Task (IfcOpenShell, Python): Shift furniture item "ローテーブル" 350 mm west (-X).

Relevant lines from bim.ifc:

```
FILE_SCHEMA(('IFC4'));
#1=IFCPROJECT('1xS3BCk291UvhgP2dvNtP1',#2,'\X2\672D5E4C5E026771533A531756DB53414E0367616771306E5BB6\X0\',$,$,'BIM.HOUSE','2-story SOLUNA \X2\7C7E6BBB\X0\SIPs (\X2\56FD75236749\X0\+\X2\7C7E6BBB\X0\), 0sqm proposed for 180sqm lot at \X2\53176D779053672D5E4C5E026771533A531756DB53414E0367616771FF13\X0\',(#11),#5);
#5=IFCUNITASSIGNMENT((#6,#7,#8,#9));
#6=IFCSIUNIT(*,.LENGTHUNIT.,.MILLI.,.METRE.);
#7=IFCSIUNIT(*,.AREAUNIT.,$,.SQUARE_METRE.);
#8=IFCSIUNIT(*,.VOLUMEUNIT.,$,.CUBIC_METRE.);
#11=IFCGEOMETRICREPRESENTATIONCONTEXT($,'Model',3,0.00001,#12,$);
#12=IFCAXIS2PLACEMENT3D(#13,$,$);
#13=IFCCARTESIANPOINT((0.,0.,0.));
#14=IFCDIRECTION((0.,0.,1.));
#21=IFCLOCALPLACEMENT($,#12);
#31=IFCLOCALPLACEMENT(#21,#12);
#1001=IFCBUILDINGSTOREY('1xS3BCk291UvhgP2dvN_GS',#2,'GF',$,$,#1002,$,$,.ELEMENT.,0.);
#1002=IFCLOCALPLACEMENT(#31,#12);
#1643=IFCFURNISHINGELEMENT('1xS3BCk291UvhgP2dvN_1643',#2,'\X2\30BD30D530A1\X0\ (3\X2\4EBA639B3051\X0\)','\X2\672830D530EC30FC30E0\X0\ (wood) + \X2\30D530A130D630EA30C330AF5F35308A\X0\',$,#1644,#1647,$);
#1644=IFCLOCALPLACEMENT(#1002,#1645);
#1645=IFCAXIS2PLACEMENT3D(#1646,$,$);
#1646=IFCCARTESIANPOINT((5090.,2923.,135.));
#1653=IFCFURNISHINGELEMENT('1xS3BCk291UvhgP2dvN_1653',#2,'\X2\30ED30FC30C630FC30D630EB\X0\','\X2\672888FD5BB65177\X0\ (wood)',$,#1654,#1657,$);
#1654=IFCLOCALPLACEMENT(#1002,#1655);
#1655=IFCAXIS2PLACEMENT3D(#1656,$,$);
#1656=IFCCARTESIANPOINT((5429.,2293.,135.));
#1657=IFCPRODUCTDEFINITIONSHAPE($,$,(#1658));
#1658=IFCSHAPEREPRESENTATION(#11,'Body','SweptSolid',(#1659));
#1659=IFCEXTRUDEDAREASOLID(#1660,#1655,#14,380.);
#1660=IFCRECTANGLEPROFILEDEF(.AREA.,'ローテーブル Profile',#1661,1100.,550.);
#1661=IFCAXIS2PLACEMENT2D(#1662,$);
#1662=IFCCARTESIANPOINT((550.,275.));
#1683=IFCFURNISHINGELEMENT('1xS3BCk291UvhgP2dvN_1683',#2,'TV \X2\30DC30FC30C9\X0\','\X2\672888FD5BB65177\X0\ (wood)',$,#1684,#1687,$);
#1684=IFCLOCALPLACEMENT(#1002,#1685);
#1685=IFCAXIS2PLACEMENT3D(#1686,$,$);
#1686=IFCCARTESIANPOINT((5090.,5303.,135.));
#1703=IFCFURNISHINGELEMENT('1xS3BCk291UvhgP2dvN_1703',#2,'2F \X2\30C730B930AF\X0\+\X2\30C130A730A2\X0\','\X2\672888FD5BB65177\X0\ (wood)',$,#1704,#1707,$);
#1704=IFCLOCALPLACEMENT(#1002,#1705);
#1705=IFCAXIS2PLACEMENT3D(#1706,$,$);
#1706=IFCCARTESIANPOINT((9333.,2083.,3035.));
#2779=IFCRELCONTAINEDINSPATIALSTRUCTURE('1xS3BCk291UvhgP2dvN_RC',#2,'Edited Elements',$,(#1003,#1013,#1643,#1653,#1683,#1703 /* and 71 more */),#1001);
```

```python
import ifcopenshell
import ifcopenshell.api.geometry
import ifcopenshell.util.placement
import ifcopenshell.util.unit

model = ifcopenshell.open("bim.ifc")
unit_scale = ifcopenshell.util.unit.calculate_unit_scale(model)

item = model.by_guid("1xS3BCk291UvhgP2dvN_1653")
matrix = ifcopenshell.util.placement.get_local_placement(item.ObjectPlacement)
matrix[0, 3] -= 0.35 / unit_scale
ifcopenshell.api.geometry.edit_object_placement(model, product=item, matrix=matrix, is_si=False)

print(ifcopenshell.util.placement.get_local_placement(item.ObjectPlacement).round(3) + 0.0)

model.write("bim_updated.ifc")
```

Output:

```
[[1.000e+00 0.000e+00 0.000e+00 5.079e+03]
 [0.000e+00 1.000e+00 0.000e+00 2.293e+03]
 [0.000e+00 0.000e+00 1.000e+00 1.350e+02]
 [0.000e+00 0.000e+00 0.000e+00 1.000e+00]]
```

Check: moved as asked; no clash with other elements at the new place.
